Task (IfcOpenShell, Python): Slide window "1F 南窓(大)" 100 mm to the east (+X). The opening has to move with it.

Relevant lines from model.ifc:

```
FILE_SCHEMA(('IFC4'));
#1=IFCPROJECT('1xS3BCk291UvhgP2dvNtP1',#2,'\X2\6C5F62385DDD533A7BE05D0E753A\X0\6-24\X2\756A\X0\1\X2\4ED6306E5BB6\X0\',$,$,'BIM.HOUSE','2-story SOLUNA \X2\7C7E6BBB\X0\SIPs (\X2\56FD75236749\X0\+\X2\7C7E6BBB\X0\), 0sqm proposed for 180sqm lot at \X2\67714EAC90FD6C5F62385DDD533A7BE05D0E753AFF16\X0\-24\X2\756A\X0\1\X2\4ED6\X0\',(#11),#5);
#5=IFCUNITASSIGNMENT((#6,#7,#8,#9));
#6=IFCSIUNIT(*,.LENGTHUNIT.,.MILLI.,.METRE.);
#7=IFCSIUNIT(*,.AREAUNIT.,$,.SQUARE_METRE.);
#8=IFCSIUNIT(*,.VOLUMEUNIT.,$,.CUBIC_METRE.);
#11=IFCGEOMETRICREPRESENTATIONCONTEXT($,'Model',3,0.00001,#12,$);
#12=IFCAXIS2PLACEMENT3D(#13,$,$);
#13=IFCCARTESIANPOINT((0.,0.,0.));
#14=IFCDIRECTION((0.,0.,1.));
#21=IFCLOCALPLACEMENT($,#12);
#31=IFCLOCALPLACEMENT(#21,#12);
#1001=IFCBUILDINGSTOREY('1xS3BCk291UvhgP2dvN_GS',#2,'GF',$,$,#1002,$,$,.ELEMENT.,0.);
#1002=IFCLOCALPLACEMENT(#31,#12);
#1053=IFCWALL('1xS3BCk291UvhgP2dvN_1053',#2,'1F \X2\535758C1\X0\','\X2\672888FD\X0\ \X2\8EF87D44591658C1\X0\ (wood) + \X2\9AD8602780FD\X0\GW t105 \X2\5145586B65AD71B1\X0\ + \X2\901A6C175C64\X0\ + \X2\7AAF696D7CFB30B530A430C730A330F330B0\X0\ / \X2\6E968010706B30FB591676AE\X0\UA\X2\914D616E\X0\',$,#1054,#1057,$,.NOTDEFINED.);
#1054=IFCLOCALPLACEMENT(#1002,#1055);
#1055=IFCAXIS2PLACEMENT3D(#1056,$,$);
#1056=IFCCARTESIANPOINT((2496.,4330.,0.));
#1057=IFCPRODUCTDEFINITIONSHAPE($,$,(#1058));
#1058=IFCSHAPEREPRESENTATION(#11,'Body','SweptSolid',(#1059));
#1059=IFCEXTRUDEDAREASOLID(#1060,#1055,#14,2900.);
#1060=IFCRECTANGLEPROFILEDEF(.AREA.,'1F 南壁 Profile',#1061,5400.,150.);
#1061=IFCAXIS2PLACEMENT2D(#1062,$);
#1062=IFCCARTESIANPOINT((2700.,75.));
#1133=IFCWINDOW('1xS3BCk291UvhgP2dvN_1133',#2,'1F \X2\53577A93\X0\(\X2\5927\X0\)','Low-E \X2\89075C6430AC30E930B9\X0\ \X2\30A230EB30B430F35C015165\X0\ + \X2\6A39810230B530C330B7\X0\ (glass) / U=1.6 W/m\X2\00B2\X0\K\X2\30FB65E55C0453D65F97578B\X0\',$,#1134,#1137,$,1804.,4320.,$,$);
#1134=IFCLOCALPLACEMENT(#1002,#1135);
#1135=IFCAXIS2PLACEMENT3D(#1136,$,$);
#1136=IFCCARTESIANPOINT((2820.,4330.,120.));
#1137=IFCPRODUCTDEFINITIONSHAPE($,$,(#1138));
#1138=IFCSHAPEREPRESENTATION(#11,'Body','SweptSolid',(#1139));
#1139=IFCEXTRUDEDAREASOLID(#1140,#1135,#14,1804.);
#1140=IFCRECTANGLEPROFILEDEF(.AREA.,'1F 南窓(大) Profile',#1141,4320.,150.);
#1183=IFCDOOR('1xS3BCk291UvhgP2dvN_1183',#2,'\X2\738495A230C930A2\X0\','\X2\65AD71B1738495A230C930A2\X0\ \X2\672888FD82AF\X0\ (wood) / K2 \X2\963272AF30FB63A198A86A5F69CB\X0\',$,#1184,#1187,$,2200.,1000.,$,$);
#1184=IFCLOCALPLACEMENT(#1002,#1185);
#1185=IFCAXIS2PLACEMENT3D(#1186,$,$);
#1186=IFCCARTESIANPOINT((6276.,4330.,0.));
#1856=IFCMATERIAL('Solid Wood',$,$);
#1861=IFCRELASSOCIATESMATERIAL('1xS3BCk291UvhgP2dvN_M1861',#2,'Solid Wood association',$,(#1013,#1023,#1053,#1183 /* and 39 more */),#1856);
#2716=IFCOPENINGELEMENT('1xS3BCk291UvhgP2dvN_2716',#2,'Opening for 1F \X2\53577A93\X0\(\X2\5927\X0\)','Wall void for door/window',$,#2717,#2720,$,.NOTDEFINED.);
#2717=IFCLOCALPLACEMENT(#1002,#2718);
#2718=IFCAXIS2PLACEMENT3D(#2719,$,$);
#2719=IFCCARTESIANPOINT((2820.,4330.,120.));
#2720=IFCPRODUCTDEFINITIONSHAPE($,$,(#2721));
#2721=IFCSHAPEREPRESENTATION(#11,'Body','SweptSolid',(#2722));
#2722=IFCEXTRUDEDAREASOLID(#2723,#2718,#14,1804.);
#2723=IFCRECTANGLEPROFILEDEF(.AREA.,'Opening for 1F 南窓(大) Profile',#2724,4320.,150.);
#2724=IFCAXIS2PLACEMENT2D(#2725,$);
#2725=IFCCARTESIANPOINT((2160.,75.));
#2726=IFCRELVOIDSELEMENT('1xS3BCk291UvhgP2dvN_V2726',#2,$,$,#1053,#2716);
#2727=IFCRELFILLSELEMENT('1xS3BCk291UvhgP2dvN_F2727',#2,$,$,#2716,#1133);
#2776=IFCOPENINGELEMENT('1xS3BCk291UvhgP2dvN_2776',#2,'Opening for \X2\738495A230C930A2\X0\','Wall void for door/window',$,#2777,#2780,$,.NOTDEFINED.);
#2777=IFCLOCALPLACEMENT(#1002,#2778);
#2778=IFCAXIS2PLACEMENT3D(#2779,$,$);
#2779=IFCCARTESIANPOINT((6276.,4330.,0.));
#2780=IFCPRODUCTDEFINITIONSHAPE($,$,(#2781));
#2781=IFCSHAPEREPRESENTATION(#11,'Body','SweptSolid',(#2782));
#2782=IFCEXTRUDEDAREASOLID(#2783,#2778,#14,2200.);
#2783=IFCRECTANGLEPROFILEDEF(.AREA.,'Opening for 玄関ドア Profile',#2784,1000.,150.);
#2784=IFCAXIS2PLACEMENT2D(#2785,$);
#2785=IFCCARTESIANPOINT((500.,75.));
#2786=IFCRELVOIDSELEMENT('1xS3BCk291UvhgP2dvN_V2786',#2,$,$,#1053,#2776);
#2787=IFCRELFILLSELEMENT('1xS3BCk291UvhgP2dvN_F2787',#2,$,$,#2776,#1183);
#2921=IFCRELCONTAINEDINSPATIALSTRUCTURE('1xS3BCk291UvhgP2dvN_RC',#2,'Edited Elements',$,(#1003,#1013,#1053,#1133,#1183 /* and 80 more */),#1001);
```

```python
import ifcopenshell
import ifcopenshell.api.geometry
import ifcopenshell.util.placement
import ifcopenshell.util.unit

model = ifcopenshell.open("model.ifc")
unit_scale = ifcopenshell.util.unit.calculate_unit_scale(model)

window = model.by_guid("1xS3BCk291UvhgP2dvN_1133")
opening = window.FillsVoids[0].RelatingOpeningElement
wall = opening.VoidsElements[0].RelatingBuildingElement

wall_matrix = ifcopenshell.util.placement.get_local_placement(wall.ObjectPlacement)
shift = wall_matrix[:3, 0] * 0.1 / unit_scale
before = ifcopenshell.util.placement.get_local_placement(window.ObjectPlacement)[:3, 3].copy()

# The window is not placed relative to its opening, so move both.
for product in (opening, window):
    matrix = ifcopenshell.util.placement.get_local_placement(product.ObjectPlacement)
    matrix[:3, 3] += shift
    ifcopenshell.api.geometry.edit_object_placement(model, product=product, matrix=matrix, is_si=False)

after = ifcopenshell.util.placement.get_local_placement(window.ObjectPlacement)[:3, 3]
print("window moved by", (after - before).round(3) + 0.0)

model.write("model_rev.ifc")
```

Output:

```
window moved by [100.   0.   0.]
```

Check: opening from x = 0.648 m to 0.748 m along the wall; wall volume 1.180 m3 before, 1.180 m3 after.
